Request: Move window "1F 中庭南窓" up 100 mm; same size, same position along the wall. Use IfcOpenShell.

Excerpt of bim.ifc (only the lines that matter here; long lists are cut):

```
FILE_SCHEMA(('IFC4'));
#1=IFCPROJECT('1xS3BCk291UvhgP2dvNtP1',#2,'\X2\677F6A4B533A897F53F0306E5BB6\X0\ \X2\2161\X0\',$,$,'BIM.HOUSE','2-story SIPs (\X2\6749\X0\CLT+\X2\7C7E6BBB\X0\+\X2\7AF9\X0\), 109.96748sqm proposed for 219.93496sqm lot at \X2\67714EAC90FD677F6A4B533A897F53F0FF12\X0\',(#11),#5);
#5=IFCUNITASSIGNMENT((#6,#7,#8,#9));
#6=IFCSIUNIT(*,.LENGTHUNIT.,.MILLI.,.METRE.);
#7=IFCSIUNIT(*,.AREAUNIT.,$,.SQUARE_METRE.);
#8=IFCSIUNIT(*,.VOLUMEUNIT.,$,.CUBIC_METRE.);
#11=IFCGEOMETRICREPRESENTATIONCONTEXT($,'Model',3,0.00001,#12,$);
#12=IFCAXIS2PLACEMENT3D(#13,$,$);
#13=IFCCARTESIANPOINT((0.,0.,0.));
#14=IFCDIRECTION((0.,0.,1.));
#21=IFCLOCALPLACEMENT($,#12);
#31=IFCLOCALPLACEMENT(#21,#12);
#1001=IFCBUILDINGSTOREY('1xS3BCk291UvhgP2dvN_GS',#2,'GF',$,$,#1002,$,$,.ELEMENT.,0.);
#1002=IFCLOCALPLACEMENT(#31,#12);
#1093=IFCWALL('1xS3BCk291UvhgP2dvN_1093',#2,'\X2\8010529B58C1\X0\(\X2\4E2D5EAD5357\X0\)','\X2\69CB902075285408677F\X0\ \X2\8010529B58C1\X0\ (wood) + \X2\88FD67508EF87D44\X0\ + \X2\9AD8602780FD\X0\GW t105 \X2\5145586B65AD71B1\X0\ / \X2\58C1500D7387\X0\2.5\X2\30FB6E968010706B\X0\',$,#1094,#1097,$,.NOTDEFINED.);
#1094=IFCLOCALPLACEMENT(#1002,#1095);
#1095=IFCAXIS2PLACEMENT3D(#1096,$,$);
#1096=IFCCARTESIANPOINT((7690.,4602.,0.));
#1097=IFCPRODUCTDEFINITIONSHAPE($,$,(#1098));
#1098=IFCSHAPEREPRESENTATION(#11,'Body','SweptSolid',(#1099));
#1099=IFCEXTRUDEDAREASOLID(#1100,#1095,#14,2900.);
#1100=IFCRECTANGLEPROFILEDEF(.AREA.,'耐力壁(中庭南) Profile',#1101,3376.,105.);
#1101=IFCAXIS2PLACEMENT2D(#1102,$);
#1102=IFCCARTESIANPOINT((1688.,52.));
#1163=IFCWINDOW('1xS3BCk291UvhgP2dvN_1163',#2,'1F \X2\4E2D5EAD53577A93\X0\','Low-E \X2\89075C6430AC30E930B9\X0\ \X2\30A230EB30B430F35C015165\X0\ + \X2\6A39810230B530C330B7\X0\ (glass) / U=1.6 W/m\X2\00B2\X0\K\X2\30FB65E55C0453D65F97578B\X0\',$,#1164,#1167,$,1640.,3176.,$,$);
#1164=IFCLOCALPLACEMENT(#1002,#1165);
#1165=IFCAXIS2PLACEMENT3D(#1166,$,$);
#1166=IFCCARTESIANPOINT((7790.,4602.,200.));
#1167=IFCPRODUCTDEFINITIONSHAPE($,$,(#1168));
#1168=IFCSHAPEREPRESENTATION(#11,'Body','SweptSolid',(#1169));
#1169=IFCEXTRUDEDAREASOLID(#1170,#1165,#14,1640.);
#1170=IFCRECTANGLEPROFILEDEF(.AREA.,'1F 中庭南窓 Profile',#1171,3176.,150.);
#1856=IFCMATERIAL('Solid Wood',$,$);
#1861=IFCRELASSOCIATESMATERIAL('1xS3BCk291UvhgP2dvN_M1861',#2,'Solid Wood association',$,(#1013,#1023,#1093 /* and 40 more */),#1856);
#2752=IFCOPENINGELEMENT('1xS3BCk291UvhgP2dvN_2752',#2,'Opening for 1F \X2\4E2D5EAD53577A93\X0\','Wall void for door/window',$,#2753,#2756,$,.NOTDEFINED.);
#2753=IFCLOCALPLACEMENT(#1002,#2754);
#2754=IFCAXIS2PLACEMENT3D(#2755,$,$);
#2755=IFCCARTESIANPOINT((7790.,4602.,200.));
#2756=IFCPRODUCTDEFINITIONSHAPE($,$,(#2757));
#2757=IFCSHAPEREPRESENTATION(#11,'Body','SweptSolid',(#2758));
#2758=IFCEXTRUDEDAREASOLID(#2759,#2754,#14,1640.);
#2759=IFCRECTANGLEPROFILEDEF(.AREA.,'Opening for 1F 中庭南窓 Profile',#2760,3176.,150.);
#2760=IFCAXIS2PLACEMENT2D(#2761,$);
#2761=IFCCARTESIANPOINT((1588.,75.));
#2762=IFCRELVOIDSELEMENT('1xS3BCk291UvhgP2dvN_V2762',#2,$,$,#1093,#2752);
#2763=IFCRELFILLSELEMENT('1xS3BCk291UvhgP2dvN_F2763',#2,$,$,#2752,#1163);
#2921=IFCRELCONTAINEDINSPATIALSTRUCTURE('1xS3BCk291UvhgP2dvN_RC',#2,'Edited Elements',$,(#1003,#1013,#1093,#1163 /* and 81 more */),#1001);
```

```python
import numpy as np
import ifcopenshell
import ifcopenshell.api.geometry
import ifcopenshell.util.placement
import ifcopenshell.util.unit

model = ifcopenshell.open("bim.ifc")
unit_scale = ifcopenshell.util.unit.calculate_unit_scale(model)

window = model.by_guid("1xS3BCk291UvhgP2dvN_1163")
opening = window.FillsVoids[0].RelatingOpeningElement
dz = 100.0

shift = np.array([0.0, 0.0, dz])
# The window is not placed relative to its opening, so move both.
for product in (opening, window):
    matrix = ifcopenshell.util.placement.get_local_placement(product.ObjectPlacement)
    matrix[:3, 3] += shift
    ifcopenshell.api.geometry.edit_object_placement(model, product=product, matrix=matrix, is_si=False)

print(f"moved by {dz * unit_scale:+.3f} m")

model.write("bim_edited.ifc")
```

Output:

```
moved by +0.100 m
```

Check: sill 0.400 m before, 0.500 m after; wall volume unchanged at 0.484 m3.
